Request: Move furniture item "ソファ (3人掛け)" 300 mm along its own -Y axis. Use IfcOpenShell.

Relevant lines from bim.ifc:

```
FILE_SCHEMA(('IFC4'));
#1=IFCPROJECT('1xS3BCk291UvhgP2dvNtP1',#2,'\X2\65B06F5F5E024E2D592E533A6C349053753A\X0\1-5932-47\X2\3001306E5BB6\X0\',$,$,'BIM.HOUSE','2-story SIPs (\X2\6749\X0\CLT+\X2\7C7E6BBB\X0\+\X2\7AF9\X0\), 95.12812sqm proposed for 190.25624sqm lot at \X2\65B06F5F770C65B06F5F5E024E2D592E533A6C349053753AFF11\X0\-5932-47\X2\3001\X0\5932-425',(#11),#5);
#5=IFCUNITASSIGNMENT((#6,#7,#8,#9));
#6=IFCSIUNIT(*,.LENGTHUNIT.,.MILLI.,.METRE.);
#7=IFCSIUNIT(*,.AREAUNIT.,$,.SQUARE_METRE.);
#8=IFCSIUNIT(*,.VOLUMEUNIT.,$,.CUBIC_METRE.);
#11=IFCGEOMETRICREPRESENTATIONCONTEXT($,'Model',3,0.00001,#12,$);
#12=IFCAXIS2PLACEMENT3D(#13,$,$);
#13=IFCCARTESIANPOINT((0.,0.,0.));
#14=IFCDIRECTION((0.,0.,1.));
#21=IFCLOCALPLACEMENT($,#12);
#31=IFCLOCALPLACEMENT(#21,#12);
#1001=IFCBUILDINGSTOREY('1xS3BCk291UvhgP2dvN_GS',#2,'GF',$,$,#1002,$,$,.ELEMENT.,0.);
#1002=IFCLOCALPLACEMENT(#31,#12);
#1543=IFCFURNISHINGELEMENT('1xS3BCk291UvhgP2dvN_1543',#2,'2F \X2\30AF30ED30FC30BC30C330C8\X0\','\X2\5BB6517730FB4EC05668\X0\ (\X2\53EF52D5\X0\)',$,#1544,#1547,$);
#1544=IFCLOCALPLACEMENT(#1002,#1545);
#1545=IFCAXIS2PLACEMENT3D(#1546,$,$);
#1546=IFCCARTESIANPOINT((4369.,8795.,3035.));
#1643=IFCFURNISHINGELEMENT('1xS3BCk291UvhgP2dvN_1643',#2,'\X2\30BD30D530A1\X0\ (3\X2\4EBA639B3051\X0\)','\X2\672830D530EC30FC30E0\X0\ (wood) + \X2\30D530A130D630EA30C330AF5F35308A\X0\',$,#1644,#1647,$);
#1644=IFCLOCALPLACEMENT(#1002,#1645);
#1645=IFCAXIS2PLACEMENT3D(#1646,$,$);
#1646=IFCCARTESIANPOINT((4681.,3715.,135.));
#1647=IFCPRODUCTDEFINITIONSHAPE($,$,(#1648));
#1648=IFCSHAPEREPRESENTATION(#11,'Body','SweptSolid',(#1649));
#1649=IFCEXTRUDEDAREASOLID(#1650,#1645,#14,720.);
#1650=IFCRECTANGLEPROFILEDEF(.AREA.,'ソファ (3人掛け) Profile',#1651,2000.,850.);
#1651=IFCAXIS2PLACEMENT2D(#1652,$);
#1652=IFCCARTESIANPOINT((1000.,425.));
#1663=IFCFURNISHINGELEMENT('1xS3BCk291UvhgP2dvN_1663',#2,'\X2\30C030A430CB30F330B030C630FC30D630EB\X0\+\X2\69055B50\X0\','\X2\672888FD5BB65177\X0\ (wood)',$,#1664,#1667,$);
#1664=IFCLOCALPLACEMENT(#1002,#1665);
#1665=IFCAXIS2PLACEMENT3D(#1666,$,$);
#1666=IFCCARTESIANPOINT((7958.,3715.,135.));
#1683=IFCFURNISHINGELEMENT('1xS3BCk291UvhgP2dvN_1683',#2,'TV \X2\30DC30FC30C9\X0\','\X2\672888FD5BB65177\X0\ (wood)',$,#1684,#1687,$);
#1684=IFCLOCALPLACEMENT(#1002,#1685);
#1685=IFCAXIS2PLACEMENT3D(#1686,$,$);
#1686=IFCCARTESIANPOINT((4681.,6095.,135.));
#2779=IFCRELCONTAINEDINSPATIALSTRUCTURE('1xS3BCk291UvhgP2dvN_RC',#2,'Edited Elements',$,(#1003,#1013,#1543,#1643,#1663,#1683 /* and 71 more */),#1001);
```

```python
import ifcopenshell
import ifcopenshell.api.geometry
import ifcopenshell.util.placement
import ifcopenshell.util.unit

model = ifcopenshell.open("bim.ifc")
unit_scale = ifcopenshell.util.unit.calculate_unit_scale(model)

item = model.by_id(1643)
matrix = ifcopenshell.util.placement.get_local_placement(item.ObjectPlacement)
matrix[:3, 3] -= matrix[:3, 1] * 0.3 / unit_scale
ifcopenshell.api.geometry.edit_object_placement(model, product=item, matrix=matrix, is_si=False)

print(ifcopenshell.util.placement.get_local_placement(item.ObjectPlacement).round(3) + 0.0)

model.write("bim_edited.ifc")
```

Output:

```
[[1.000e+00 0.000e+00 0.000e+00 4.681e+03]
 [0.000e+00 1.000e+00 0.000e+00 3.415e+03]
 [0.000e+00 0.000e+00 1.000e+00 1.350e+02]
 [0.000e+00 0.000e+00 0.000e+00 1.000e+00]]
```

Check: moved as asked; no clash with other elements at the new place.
